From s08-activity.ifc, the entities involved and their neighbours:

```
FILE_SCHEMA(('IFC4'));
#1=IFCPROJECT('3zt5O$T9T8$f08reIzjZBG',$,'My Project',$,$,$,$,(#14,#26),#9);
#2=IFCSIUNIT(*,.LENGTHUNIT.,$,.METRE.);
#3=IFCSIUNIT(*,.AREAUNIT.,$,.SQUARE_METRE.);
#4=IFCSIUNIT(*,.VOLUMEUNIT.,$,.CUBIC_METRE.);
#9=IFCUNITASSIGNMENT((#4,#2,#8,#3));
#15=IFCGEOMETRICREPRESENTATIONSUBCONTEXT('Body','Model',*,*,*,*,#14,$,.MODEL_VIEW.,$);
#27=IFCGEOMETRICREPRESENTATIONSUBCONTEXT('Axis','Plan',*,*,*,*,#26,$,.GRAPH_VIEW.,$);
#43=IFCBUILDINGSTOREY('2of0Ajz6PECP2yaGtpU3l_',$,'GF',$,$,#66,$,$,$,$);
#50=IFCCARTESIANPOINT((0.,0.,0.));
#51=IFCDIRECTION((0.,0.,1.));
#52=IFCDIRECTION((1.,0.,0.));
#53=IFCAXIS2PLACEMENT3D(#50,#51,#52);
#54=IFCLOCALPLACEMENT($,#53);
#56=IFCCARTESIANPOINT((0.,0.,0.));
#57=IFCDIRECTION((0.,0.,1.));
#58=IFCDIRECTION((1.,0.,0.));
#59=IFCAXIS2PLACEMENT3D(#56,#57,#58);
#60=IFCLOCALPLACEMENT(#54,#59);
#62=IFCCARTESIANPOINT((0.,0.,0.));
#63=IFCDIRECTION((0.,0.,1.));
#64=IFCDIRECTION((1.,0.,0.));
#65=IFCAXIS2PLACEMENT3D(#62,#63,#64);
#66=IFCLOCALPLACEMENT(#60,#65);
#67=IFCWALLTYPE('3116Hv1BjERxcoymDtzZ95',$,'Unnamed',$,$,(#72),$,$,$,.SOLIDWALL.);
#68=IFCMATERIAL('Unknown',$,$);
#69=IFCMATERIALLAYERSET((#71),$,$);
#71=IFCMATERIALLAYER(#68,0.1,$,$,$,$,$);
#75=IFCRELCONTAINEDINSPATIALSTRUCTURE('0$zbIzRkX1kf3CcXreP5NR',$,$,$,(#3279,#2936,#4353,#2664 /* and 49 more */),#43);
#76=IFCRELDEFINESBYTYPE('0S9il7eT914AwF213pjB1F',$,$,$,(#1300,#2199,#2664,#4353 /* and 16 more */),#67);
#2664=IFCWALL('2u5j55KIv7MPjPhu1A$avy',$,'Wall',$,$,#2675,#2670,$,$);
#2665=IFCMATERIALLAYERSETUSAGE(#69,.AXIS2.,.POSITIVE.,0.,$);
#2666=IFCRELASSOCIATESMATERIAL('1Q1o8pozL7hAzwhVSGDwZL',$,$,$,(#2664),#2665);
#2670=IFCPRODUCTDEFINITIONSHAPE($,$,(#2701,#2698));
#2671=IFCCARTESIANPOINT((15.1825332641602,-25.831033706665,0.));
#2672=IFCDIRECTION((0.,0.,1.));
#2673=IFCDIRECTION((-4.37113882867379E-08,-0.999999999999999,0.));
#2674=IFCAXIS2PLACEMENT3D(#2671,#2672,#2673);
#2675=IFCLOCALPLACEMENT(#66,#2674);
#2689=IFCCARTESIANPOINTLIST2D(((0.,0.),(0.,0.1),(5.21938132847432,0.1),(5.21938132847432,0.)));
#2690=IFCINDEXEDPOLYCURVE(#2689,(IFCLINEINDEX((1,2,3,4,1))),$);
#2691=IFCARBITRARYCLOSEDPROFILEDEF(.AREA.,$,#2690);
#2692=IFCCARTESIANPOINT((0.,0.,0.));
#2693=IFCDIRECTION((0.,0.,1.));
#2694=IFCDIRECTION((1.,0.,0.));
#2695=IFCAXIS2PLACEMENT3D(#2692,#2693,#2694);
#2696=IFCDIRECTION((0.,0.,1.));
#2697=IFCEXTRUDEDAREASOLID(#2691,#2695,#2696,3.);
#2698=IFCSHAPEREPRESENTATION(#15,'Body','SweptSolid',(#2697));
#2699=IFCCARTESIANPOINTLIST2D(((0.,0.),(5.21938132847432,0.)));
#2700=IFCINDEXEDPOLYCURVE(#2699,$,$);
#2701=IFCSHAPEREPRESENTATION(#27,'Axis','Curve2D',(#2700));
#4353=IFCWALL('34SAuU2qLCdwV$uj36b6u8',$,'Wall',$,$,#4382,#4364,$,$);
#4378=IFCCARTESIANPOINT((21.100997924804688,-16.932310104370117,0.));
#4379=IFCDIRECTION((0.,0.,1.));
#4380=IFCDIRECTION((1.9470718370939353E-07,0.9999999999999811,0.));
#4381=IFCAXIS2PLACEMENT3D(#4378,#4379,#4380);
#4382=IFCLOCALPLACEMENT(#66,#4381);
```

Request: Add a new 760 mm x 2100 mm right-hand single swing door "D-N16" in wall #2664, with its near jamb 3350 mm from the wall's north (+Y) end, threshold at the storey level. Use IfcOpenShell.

```python
import numpy as np
import ifcopenshell
import ifcopenshell.api.feature
import ifcopenshell.api.geometry
import ifcopenshell.api.root
import ifcopenshell.api.spatial
import ifcopenshell.geom
import ifcopenshell.util.element
import ifcopenshell.util.placement
import ifcopenshell.util.representation
import ifcopenshell.util.shape
import ifcopenshell.util.unit

model = ifcopenshell.open("s08-activity.ifc")
unit_scale = ifcopenshell.util.unit.calculate_unit_scale(model)
settings = ifcopenshell.geom.settings()


def volume(element):
    """Net volume in cubic metres, openings subtracted."""
    shape = ifcopenshell.geom.create_shape(settings, element)
    return ifcopenshell.util.shape.get_volume(shape.geometry)


wall = model.by_id(2664)
storey = ifcopenshell.util.element.get_container(wall, ifc_class="IfcBuildingStorey")
context = ifcopenshell.util.representation.get_context(model, "Model", "Body", "MODEL_VIEW")
before = volume(wall)

width, height, from_end, sill = 0.76, 2.1, 3.35, 0.0  # metres

# The wall runs along its own X axis, and the end named is its -X end.
wall_shape = ifcopenshell.geom.create_shape(settings, wall)
x, y, z = ifcopenshell.util.shape.get_vertices(wall_shape.geometry).T
start = x.min() + from_end
face, thickness = float(y.min()), float(y.max() - y.min())
wall_matrix = ifcopenshell.util.placement.get_local_placement(wall.ObjectPlacement)
level = ifcopenshell.util.placement.get_local_placement(storey.ObjectPlacement)[2, 3]


def in_wall(x, y):
    """Placement at x, y metres in the wall's axes, at sill height."""
    matrix = wall_matrix.copy()
    matrix[:, 3] = wall_matrix @ np.array([x / unit_scale, y / unit_scale, 0.0, 1.0])
    matrix[2, 3] = level + sill / unit_scale
    return matrix


# Opening: a box that overshoots both wall faces by 50 mm.
opening = ifcopenshell.api.root.create_entity(model, ifc_class="IfcOpeningElement", predefined_type="OPENING")
box = ifcopenshell.api.geometry.add_wall_representation(
    model, context=context, length=width, height=height, thickness=thickness + 0.1
)
ifcopenshell.api.geometry.assign_representation(model, product=opening, representation=box)
ifcopenshell.api.geometry.edit_object_placement(model, product=opening, matrix=in_wall(start, face - 0.05), is_si=False)
ifcopenshell.api.feature.add_feature(model, feature=opening, element=wall)

door = ifcopenshell.api.root.create_entity(model, ifc_class="IfcDoor", name="D-N16", predefined_type="DOOR")
door.OverallWidth, door.OverallHeight = width / unit_scale, height / unit_scale
door.OperationType = "SINGLE_SWING_RIGHT"
body = ifcopenshell.api.geometry.add_door_representation(
    model,
    context=context,
    overall_width=door.OverallWidth,
    overall_height=door.OverallHeight,
    operation_type="SINGLE_SWING_RIGHT",
    lining_properties={"LiningDepth": thickness / unit_scale, "ThresholdDepth": thickness / unit_scale},
)
ifcopenshell.api.geometry.assign_representation(model, product=door, representation=body)
ifcopenshell.api.spatial.assign_container(model, products=[door], relating_structure=storey)
ifcopenshell.api.feature.add_filling(model, opening=opening, element=door)

# The lining spans the wall, so the door starts at the wall face.
ifcopenshell.api.geometry.edit_object_placement(model, product=door, matrix=in_wall(start, face), is_si=False)

after = volume(wall)

print(f"wall volume {before:.3f} -> {after:.3f} m3")

model.write("s08-activity_v2.ifc")
```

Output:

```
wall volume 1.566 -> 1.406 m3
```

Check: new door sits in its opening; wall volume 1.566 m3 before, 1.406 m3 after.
